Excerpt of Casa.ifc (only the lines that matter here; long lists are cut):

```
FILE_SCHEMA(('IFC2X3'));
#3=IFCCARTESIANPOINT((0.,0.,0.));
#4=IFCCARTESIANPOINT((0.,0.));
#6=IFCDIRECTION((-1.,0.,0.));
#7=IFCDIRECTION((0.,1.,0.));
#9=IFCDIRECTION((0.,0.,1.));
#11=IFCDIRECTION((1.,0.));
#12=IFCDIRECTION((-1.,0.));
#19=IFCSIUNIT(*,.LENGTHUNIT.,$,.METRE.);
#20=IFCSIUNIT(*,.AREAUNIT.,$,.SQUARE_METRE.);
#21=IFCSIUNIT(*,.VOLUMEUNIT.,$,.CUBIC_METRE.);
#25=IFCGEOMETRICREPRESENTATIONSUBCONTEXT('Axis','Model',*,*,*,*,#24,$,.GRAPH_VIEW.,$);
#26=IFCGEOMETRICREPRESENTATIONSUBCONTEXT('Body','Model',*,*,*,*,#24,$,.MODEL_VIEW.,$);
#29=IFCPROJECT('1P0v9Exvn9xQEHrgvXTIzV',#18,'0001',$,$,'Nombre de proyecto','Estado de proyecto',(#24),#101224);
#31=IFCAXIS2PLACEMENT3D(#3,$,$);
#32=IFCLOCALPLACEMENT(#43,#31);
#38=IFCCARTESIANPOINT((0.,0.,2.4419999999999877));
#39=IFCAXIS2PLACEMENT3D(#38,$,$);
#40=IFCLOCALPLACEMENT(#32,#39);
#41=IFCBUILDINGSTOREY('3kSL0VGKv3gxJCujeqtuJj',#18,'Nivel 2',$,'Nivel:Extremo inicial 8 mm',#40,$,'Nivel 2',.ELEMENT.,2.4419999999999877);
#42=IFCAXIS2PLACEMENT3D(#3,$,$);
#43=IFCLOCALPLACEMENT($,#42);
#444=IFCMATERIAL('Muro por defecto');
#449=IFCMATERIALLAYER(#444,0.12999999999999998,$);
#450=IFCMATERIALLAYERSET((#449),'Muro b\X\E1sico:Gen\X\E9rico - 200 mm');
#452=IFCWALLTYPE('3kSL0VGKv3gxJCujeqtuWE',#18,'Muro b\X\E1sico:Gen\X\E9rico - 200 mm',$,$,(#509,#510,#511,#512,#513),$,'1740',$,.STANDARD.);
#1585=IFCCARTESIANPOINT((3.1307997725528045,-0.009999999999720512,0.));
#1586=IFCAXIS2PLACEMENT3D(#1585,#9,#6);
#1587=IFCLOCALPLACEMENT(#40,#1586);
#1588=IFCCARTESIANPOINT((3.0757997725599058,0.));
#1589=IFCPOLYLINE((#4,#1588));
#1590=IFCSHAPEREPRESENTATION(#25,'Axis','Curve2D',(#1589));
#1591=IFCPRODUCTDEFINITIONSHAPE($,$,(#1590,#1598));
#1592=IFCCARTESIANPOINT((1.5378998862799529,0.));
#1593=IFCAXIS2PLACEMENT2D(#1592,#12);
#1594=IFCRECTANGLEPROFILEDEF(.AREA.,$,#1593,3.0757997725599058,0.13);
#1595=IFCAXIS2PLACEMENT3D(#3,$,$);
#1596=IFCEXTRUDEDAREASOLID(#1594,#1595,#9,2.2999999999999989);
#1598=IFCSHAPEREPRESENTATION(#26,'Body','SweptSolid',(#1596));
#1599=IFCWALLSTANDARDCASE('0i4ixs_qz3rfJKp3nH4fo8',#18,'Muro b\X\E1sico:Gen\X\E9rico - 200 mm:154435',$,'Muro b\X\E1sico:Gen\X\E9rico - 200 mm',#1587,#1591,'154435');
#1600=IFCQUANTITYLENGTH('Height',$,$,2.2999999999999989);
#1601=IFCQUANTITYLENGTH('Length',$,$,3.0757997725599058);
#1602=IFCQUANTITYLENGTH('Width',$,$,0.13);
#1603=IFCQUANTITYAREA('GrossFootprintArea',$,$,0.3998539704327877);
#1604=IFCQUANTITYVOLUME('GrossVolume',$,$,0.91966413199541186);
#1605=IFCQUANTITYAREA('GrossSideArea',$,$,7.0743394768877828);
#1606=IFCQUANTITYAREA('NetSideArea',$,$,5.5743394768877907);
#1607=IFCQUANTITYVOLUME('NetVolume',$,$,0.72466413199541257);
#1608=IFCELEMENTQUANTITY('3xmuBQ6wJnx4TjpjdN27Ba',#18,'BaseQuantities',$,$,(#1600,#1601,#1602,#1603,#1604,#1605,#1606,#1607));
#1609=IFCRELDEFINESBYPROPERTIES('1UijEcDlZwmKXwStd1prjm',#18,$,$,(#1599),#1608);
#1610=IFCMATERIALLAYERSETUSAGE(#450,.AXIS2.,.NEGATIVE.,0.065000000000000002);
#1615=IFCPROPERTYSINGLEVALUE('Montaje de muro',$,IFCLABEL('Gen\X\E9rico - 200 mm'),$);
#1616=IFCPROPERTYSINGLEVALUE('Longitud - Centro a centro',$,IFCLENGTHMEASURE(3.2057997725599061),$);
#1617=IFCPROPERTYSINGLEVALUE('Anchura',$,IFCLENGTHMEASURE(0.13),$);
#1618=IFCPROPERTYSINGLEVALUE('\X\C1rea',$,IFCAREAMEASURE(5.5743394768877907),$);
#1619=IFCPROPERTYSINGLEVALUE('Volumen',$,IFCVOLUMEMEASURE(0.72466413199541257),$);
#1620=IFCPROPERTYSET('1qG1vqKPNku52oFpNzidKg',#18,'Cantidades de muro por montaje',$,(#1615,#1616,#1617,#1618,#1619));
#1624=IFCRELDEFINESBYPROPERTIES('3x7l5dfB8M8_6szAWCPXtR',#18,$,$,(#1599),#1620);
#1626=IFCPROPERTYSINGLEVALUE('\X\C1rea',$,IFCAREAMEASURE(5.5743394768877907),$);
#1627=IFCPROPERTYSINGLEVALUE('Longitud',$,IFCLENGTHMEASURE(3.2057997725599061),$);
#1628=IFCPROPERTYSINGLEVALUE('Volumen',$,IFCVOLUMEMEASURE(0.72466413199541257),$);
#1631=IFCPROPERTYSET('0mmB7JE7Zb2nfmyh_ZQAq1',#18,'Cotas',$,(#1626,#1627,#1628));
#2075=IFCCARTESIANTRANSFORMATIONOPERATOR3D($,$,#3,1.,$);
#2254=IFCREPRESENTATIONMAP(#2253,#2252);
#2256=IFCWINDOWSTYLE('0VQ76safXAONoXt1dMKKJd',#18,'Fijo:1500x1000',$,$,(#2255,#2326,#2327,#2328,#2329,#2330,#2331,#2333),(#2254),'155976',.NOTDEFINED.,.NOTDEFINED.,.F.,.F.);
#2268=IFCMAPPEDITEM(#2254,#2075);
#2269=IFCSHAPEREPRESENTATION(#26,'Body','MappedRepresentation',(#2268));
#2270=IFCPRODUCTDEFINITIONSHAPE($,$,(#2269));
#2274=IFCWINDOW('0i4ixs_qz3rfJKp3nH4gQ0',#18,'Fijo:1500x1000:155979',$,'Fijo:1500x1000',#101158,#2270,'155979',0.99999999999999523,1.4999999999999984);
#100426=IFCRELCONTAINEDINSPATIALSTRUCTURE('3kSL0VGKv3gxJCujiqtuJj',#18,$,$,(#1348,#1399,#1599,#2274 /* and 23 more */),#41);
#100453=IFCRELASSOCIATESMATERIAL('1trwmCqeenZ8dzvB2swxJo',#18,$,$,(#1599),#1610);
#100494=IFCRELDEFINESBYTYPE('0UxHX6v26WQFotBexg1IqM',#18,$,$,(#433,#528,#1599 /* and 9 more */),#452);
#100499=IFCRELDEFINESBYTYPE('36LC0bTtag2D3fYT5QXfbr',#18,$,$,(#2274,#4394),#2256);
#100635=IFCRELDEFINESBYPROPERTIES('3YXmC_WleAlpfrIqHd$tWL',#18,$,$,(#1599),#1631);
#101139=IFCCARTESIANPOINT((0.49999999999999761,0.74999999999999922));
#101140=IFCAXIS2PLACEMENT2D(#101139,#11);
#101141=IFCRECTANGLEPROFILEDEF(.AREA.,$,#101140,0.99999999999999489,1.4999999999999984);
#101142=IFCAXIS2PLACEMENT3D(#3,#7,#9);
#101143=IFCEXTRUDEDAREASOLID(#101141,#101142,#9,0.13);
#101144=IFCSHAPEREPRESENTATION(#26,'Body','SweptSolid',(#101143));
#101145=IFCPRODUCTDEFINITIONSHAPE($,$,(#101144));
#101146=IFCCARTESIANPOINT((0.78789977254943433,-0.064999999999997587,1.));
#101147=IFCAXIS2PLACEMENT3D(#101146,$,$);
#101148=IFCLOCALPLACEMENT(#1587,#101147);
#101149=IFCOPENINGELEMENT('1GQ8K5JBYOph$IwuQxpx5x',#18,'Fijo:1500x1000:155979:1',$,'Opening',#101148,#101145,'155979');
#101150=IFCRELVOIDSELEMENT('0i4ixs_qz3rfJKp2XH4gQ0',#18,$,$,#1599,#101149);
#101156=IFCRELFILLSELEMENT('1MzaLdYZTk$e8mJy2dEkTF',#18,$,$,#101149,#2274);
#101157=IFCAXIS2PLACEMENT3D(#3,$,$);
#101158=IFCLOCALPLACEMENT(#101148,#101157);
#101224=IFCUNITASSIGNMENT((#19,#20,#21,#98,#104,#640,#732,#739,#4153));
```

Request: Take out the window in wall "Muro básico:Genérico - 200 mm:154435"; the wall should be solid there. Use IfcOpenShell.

```python
import ifcopenshell
import ifcopenshell.api.feature
import ifcopenshell.api.pset
import ifcopenshell.api.root
import ifcopenshell.geom
import ifcopenshell.util.element
import ifcopenshell.util.shape
import ifcopenshell.util.unit

model = ifcopenshell.open("Casa.ifc")
area_scale = ifcopenshell.util.unit.calculate_unit_scale(model, "AREAUNIT")
volume_scale = ifcopenshell.util.unit.calculate_unit_scale(model, "VOLUMEUNIT")
settings = ifcopenshell.geom.settings()


def volume(element):
    """Net volume in cubic metres, openings subtracted."""
    shape = ifcopenshell.geom.create_shape(settings, element)
    return ifcopenshell.util.shape.get_volume(shape.geometry)


window = model.by_guid("0i4ixs_qz3rfJKp3nH4gQ0")
opening = window.FillsVoids[0].RelatingOpeningElement
wall = opening.VoidsElements[0].RelatingBuildingElement
before = volume(wall)

ifcopenshell.api.root.remove_product(model, product=window)
ifcopenshell.api.feature.remove_feature(model, feature=opening)

after = volume(wall)
thickness = 0.13  # wall thickness in metres

# Update the wall's stored quantities.
qto = model.by_id(ifcopenshell.util.element.get_pset(wall, "BaseQuantities", should_inherit=False)["id"])
ifcopenshell.api.pset.edit_qto(model, qto=qto, properties={
    "NetSideArea": after / thickness / area_scale,
    "NetVolume": after / volume_scale,
})
pset = model.by_id(ifcopenshell.util.element.get_pset(wall, "Cantidades de muro por montaje", should_inherit=False)["id"])
ifcopenshell.api.pset.edit_pset(model, pset=pset, properties={
    "Área": model.create_entity("IfcAreaMeasure", after / thickness / area_scale),
    "Volumen": model.create_entity("IfcVolumeMeasure", after / volume_scale),
})
pset = model.by_id(ifcopenshell.util.element.get_pset(wall, "Cotas", should_inherit=False)["id"])
ifcopenshell.api.pset.edit_pset(model, pset=pset, properties={
    "Área": model.create_entity("IfcAreaMeasure", after / thickness / area_scale),
    "Volumen": model.create_entity("IfcVolumeMeasure", after / volume_scale),
})

print(f"wall volume {before:.3f} -> {after:.3f} m3")

model.write("Casa_v2.ifc")
```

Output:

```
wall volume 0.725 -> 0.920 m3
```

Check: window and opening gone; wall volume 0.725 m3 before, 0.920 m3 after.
